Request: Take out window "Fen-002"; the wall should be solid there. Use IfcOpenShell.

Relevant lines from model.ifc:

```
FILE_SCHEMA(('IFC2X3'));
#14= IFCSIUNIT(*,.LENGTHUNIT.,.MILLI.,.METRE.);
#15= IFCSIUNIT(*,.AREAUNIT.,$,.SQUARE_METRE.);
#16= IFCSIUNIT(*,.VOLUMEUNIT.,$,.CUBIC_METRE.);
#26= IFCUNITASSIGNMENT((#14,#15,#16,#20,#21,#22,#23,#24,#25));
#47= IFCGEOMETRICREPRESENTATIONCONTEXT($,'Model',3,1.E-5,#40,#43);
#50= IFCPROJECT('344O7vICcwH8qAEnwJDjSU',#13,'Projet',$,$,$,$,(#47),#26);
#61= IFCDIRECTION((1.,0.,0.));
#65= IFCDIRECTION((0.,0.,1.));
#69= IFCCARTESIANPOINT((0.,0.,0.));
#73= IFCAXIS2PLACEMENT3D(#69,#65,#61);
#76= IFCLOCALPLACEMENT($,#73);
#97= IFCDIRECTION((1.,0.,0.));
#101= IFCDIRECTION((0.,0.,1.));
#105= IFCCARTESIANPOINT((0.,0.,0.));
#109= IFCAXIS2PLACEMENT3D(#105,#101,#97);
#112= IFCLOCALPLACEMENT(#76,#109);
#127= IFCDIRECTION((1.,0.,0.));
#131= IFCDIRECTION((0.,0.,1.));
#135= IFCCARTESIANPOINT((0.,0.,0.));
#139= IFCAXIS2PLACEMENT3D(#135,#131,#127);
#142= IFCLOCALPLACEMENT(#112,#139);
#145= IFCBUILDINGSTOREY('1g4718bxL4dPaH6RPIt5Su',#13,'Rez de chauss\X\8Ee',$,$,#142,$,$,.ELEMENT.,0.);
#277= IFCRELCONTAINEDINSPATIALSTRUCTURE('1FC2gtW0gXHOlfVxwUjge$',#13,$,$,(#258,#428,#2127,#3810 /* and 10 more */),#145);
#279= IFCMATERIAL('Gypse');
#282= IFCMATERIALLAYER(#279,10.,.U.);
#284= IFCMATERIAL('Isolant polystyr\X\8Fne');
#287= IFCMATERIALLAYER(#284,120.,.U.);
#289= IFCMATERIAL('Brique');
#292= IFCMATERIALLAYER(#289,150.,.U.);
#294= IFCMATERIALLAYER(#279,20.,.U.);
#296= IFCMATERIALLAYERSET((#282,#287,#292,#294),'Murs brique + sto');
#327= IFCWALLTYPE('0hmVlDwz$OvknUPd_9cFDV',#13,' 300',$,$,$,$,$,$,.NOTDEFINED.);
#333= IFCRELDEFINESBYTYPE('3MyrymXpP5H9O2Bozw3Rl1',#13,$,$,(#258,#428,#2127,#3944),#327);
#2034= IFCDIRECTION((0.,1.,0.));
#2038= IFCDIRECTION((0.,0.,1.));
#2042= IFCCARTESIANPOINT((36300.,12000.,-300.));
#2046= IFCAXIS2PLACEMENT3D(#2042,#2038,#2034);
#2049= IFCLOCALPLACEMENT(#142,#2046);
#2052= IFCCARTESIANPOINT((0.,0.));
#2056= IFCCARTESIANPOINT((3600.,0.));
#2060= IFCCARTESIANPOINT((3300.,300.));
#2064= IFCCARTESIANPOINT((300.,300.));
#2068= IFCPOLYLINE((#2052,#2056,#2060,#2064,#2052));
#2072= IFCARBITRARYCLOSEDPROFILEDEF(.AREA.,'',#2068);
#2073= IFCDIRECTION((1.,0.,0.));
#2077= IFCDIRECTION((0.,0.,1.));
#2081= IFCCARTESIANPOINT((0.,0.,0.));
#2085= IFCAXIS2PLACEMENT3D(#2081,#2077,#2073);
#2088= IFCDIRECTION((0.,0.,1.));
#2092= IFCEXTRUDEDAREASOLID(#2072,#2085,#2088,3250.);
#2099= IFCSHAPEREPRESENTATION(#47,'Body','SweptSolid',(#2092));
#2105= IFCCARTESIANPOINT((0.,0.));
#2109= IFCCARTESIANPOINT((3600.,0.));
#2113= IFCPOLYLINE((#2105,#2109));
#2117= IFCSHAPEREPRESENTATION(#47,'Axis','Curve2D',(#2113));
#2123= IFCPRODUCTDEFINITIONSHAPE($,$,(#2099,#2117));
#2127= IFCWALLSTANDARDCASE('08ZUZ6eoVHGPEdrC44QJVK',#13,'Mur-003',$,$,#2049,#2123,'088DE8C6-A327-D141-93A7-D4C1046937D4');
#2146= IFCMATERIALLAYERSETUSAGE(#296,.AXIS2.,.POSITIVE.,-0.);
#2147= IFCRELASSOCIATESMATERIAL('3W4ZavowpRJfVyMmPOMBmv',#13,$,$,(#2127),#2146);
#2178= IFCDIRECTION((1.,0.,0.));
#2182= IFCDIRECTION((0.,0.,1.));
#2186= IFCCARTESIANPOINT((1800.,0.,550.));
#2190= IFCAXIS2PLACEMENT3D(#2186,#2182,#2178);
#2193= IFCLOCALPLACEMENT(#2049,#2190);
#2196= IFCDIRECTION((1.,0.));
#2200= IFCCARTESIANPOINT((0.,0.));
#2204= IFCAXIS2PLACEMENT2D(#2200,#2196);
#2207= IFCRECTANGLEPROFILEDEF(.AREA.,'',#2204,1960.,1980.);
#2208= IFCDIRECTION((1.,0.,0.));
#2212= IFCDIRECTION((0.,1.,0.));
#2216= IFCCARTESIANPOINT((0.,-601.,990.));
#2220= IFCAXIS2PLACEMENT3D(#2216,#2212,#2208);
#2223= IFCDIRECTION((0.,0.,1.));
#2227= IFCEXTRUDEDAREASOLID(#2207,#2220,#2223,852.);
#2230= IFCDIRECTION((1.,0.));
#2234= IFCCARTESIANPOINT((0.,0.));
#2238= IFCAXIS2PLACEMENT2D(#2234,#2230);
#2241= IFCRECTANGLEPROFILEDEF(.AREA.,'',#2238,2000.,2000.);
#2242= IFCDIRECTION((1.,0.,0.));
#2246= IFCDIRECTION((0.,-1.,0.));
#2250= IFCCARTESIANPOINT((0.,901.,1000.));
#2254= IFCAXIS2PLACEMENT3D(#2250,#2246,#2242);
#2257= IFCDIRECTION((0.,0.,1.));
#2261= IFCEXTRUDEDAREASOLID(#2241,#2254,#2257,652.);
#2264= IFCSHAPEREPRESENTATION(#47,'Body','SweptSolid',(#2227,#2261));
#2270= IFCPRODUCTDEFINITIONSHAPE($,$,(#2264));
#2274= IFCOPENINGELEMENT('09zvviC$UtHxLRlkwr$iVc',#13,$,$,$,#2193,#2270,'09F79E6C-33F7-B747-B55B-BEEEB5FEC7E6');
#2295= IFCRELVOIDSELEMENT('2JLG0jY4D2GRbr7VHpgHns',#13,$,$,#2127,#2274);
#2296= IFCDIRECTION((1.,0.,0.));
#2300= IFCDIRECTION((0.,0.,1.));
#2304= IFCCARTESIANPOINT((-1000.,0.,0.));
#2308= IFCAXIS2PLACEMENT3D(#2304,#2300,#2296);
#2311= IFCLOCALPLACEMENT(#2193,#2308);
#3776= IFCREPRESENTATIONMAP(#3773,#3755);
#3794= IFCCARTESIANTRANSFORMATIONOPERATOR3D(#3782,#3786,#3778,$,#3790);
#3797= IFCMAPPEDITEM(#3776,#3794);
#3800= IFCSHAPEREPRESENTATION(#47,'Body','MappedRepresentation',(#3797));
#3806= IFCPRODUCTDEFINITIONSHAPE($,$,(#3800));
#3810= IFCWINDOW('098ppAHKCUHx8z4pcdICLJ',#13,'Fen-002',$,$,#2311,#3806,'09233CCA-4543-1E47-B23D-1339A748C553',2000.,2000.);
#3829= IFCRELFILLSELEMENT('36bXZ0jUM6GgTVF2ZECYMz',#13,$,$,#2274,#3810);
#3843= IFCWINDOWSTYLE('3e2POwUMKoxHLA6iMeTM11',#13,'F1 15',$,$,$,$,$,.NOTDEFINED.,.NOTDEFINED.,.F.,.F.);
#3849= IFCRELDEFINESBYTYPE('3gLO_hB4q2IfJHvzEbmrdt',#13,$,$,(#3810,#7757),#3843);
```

```python
import ifcopenshell
import ifcopenshell.api.feature
import ifcopenshell.api.root
import ifcopenshell.geom
import ifcopenshell.util.shape

model = ifcopenshell.open("model.ifc")
settings = ifcopenshell.geom.settings()


def volume(element):
    """Net volume in cubic metres, openings subtracted."""
    shape = ifcopenshell.geom.create_shape(settings, element)
    return ifcopenshell.util.shape.get_volume(shape.geometry)


window = model.by_guid("098ppAHKCUHx8z4pcdICLJ")
opening = window.FillsVoids[0].RelatingOpeningElement
wall = opening.VoidsElements[0].RelatingBuildingElement
before = volume(wall)

ifcopenshell.api.root.remove_product(model, product=window)
ifcopenshell.api.feature.remove_feature(model, feature=opening)

after = volume(wall)

print(f"wall volume {before:.3f} -> {after:.3f} m3")

model.write("model_v2.ifc")
```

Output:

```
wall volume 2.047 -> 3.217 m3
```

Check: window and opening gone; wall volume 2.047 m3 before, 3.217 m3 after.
